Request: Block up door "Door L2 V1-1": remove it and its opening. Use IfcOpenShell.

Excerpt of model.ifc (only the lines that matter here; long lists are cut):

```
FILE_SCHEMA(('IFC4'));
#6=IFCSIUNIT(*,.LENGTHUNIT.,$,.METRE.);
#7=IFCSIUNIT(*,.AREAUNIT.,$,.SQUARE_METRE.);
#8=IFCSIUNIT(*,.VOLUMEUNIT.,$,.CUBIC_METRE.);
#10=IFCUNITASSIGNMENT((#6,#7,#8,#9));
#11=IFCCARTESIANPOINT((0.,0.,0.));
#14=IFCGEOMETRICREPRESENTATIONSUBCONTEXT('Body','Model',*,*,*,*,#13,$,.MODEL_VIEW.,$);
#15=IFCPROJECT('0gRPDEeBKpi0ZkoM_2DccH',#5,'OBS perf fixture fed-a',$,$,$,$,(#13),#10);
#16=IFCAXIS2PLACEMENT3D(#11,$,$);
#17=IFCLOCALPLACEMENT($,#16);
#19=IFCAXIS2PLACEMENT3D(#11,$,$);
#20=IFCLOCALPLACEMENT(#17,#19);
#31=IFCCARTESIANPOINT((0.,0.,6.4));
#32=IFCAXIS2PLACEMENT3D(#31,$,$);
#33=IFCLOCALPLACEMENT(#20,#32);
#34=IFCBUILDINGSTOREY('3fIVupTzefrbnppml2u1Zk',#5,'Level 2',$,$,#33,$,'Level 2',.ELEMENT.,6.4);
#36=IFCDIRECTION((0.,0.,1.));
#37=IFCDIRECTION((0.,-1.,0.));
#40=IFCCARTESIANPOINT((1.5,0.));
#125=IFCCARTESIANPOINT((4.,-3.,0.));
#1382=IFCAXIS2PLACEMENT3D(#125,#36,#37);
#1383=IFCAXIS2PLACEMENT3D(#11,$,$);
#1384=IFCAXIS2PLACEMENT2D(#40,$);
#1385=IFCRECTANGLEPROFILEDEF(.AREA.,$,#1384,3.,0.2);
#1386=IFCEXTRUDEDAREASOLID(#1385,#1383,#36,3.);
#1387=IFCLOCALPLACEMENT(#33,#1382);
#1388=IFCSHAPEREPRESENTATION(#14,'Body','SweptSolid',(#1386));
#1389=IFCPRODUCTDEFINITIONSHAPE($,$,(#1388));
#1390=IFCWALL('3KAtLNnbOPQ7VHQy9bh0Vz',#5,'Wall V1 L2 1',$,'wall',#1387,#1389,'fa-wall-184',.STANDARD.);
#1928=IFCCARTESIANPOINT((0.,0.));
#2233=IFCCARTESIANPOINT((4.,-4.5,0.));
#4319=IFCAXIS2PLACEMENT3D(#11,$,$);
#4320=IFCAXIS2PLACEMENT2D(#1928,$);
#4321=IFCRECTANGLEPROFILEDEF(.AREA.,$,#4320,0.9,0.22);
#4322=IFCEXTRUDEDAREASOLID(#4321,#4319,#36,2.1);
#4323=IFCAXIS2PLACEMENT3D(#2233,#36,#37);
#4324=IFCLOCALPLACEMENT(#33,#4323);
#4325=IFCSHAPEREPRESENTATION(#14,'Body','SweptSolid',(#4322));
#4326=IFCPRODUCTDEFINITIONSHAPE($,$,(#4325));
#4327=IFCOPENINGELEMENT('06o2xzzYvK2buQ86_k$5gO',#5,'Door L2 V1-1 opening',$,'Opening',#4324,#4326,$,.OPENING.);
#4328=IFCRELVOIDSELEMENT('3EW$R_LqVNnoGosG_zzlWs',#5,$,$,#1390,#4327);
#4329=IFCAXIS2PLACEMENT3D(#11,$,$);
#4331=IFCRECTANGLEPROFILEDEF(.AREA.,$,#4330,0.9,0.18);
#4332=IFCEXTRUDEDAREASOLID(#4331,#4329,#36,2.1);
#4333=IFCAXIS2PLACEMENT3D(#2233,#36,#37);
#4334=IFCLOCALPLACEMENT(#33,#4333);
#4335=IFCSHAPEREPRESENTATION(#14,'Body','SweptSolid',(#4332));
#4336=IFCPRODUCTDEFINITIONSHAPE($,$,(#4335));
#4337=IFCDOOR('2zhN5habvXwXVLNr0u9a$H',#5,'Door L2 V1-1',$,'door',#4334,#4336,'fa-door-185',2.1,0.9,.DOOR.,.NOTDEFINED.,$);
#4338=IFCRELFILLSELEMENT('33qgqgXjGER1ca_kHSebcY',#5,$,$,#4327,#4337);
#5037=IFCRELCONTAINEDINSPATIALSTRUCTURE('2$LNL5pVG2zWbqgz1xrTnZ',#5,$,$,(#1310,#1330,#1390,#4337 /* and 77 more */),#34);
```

```python
import ifcopenshell
import ifcopenshell.api.feature
import ifcopenshell.api.root
import ifcopenshell.geom
import ifcopenshell.util.shape

model = ifcopenshell.open("model.ifc")
settings = ifcopenshell.geom.settings()


def volume(element):
    """Net volume in cubic metres, openings subtracted."""
    shape = ifcopenshell.geom.create_shape(settings, element)
    return ifcopenshell.util.shape.get_volume(shape.geometry)


door = model.by_id(4337)
opening = door.FillsVoids[0].RelatingOpeningElement
wall = opening.VoidsElements[0].RelatingBuildingElement
before = volume(wall)

ifcopenshell.api.root.remove_product(model, product=door)
ifcopenshell.api.feature.remove_feature(model, feature=opening)

after = volume(wall)

print(f"wall volume {before:.3f} -> {after:.3f} m3")

model.write("model_updated.ifc")
```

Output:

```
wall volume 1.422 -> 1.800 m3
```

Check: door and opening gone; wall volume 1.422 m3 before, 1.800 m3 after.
